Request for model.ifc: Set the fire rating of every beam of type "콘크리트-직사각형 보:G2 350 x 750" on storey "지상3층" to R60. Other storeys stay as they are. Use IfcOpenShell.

First a look at what the model holds.

```python
import ifcopenshell
import ifcopenshell.util.element

model = ifcopenshell.open("model.ifc")
print(model.schema)
storey = next(s for s in model.by_type("IfcBuildingStorey") if s.Name == "지상3층")
beams = [e for e in ifcopenshell.util.element.get_decomposition(storey) if e.is_a("IfcBeam")]
seen = {}
for e in beams:
    element_type = ifcopenshell.util.element.get_type(e)
    key = (element_type.Name if element_type != e and element_type else None, ifcopenshell.util.element.get_pset(e, "Pset_BeamCommon", "FireRating"))
    seen[key] = seen.get(key, 0) + 1
for (name, value), count in sorted(seen.items(), key=str):
    print(count, "x", name, "|", value)
```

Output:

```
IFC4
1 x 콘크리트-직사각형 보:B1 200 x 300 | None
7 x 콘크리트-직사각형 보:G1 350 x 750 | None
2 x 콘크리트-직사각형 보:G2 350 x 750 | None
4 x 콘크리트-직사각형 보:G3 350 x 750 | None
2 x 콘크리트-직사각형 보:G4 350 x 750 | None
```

```python
import ifcopenshell
import ifcopenshell.api.pset
import ifcopenshell.util.element

model = ifcopenshell.open("model.ifc")

storey = next(s for s in model.by_type("IfcBuildingStorey") if s.Name == "지상3층")
beams = [e for e in ifcopenshell.util.element.get_decomposition(storey) if e.is_a("IfcBeam")]

count = 0
for e in beams:
    element_type = ifcopenshell.util.element.get_type(e)
    if element_type in (None, e) or element_type.Name != "콘크리트-직사각형 보:G2 350 x 750":
        continue
    # add_pset returns the element's existing set when there is one.
    pset = ifcopenshell.api.pset.add_pset(model, product=e, name="Pset_BeamCommon")
    ifcopenshell.api.pset.edit_pset(model, pset=pset, properties={"FireRating": "R60"})
    count += 1

print(count, "beams updated")

model.write("model_rev.ifc")
```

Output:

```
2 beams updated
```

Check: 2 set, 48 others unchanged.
